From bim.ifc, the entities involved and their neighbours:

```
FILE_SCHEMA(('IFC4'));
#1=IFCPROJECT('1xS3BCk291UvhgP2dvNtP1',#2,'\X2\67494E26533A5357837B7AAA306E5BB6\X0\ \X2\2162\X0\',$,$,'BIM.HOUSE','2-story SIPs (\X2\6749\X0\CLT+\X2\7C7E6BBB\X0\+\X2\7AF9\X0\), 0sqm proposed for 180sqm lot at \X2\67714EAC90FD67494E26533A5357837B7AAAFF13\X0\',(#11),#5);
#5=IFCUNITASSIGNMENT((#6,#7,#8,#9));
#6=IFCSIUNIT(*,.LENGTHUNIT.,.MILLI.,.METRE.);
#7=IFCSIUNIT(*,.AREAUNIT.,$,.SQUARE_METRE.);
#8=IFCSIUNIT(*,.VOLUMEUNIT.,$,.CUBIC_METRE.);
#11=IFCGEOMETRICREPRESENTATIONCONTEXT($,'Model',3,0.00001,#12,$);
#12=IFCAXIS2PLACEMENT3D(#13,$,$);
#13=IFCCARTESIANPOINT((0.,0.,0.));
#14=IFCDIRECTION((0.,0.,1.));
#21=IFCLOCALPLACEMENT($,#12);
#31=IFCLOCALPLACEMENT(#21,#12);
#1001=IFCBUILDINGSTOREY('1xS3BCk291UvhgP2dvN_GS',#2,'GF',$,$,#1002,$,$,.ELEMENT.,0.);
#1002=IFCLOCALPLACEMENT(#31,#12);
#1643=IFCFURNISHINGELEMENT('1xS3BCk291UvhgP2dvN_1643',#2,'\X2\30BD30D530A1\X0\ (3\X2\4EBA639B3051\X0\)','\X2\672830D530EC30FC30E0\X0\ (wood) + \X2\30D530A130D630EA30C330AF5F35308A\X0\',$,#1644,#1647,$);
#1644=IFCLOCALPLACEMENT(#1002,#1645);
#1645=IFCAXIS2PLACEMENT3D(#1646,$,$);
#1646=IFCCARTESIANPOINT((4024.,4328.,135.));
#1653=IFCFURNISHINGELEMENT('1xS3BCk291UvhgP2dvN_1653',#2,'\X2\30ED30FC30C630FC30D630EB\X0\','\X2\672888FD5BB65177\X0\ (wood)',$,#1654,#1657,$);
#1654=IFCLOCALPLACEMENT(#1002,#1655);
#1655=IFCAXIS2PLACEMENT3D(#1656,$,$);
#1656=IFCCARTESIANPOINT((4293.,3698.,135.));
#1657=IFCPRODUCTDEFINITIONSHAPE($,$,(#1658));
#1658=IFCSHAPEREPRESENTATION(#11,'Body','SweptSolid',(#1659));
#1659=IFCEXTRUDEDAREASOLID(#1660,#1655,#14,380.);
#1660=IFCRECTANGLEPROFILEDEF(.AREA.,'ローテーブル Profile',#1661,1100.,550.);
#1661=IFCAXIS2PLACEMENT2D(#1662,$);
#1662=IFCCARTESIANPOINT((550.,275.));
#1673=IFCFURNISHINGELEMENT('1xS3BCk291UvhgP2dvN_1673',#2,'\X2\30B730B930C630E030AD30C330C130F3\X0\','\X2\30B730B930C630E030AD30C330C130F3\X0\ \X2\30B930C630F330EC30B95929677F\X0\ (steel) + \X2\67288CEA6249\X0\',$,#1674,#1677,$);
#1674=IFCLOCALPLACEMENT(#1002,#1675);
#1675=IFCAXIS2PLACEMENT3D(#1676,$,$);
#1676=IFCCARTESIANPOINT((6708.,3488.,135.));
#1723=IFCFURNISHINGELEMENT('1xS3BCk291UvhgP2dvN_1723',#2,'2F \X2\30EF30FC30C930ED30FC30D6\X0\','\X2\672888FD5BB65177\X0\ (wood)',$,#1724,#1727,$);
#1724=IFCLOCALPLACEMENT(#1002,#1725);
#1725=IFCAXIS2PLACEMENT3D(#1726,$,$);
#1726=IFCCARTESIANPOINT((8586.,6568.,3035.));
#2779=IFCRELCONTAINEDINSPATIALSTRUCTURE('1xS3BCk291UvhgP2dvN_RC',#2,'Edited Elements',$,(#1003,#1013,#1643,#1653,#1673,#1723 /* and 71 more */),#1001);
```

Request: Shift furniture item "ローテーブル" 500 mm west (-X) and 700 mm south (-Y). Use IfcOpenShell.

```python
import ifcopenshell
import ifcopenshell.api.geometry
import ifcopenshell.util.placement

model = ifcopenshell.open("bim.ifc")

item = model.by_guid("1xS3BCk291UvhgP2dvN_1653")
matrix = ifcopenshell.util.placement.get_local_placement(item.ObjectPlacement)
matrix[0, 3] -= 500.0
matrix[1, 3] -= 700.0
ifcopenshell.api.geometry.edit_object_placement(model, product=item, matrix=matrix, is_si=False)

print(ifcopenshell.util.placement.get_local_placement(item.ObjectPlacement).round(3) + 0.0)

model.write("bim-out.ifc")
```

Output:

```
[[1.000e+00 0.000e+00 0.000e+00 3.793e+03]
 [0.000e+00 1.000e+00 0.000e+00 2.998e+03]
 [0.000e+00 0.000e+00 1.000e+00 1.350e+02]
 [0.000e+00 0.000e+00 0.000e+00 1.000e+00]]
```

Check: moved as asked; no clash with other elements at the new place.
